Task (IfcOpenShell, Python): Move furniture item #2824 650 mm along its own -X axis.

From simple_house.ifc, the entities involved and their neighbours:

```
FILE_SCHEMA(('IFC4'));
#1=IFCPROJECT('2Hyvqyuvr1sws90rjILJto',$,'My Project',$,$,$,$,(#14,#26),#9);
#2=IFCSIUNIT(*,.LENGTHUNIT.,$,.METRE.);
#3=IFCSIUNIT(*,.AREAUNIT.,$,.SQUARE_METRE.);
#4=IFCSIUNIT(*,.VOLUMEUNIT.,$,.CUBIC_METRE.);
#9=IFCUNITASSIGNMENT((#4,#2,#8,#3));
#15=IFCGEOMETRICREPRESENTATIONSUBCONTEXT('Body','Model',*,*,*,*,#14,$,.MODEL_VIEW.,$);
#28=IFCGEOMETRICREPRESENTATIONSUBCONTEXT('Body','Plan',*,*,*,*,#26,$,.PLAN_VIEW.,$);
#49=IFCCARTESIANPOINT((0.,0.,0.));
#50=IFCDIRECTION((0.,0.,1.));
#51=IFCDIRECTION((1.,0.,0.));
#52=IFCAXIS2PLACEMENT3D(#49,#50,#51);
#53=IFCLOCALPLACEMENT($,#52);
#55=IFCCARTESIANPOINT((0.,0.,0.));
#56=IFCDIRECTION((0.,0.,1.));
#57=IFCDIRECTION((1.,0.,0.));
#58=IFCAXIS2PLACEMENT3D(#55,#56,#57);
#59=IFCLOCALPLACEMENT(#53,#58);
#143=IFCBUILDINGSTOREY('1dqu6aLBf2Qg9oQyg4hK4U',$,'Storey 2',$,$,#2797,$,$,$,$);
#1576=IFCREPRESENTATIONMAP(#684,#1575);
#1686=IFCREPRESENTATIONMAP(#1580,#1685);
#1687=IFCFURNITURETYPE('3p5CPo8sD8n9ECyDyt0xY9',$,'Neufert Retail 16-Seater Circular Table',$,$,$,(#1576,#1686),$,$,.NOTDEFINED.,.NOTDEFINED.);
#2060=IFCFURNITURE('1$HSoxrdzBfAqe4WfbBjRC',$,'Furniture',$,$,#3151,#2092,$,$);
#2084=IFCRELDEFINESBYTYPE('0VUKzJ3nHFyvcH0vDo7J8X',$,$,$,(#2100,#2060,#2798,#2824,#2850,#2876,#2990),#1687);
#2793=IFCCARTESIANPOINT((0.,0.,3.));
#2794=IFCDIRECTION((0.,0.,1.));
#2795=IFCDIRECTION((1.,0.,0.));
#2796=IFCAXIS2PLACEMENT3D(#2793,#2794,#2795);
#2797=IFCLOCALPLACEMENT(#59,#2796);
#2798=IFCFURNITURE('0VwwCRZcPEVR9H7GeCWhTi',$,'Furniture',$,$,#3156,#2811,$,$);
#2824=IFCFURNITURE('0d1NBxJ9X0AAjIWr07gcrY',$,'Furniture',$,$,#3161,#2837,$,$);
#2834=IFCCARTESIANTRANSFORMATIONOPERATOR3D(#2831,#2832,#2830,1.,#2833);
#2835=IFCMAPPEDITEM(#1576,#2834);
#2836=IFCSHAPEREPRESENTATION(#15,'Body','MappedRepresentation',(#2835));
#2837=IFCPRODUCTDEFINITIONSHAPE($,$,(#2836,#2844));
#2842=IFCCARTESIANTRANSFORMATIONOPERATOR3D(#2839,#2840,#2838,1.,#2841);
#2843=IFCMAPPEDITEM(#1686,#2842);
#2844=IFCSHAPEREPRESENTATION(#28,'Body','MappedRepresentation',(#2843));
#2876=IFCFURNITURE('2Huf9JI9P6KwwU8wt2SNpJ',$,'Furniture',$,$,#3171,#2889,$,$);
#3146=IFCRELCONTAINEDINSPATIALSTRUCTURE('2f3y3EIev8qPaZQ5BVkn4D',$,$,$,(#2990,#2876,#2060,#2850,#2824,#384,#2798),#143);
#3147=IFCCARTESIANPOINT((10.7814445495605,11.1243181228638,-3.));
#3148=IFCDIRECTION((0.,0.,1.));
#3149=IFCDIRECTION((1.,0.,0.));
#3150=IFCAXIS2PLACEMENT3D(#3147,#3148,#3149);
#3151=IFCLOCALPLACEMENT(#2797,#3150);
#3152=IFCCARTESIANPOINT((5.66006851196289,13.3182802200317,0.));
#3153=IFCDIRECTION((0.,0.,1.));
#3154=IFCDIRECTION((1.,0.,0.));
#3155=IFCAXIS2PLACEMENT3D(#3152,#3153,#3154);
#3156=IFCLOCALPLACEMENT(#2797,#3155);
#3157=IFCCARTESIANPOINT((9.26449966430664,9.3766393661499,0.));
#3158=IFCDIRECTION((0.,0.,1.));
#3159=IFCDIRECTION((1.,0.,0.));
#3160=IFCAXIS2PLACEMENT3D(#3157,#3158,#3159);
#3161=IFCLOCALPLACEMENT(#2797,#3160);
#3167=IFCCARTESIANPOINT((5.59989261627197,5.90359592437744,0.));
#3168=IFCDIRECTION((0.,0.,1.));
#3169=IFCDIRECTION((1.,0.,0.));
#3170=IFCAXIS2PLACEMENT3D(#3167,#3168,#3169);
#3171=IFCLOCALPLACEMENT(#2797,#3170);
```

```python
import ifcopenshell
import ifcopenshell.api.geometry
import ifcopenshell.util.placement
import ifcopenshell.util.unit

model = ifcopenshell.open("simple_house.ifc")
unit_scale = ifcopenshell.util.unit.calculate_unit_scale(model)

item = model.by_guid("0d1NBxJ9X0AAjIWr07gcrY")
matrix = ifcopenshell.util.placement.get_local_placement(item.ObjectPlacement)
matrix[:3, 3] -= matrix[:3, 0] * 0.65 / unit_scale
ifcopenshell.api.geometry.edit_object_placement(model, product=item, matrix=matrix, is_si=False)

print(ifcopenshell.util.placement.get_local_placement(item.ObjectPlacement).round(3) + 0.0)

model.write("simple_house_rev.ifc")
```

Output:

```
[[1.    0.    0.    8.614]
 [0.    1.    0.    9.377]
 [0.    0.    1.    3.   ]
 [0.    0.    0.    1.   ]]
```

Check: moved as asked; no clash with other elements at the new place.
